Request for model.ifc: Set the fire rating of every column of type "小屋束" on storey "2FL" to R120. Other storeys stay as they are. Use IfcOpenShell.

First a look at what the model holds.

```python
import ifcopenshell
import ifcopenshell.util.element

model = ifcopenshell.open("model.ifc")
print(model.schema)
storey = next(s for s in model.by_type("IfcBuildingStorey") if s.Name == "2FL")
columns = [e for e in ifcopenshell.util.element.get_decomposition(storey) if e.is_a("IfcColumn")]
seen = {}
for e in columns:
    element_type = ifcopenshell.util.element.get_type(e)
    key = (element_type.Name if element_type != e and element_type else None, ifcopenshell.util.element.get_pset(e, "Pset_ColumnCommon", "FireRating"))
    seen[key] = seen.get(key, 0) + 1
for (name, value), count in sorted(seen.items(), key=str):
    print(count, "x", name, "|", value)
```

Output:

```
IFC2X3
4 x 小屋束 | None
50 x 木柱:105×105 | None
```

```python
import ifcopenshell
import ifcopenshell.api.pset
import ifcopenshell.util.element

model = ifcopenshell.open("model.ifc")

storey = next(s for s in model.by_type("IfcBuildingStorey") if s.Name == "2FL")
columns = [e for e in ifcopenshell.util.element.get_decomposition(storey) if e.is_a("IfcColumn")]

count = 0
for e in columns:
    element_type = ifcopenshell.util.element.get_type(e)
    if element_type in (None, e) or element_type.Name != "小屋束":
        continue
    # add_pset returns the element's existing set when there is one.
    pset = ifcopenshell.api.pset.add_pset(model, product=e, name="Pset_ColumnCommon")
    ifcopenshell.api.pset.edit_pset(model, pset=pset, properties={"FireRating": "R120"})
    count += 1

print(count, "columns updated")

model.write("model-out.ifc")
```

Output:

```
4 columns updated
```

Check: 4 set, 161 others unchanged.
